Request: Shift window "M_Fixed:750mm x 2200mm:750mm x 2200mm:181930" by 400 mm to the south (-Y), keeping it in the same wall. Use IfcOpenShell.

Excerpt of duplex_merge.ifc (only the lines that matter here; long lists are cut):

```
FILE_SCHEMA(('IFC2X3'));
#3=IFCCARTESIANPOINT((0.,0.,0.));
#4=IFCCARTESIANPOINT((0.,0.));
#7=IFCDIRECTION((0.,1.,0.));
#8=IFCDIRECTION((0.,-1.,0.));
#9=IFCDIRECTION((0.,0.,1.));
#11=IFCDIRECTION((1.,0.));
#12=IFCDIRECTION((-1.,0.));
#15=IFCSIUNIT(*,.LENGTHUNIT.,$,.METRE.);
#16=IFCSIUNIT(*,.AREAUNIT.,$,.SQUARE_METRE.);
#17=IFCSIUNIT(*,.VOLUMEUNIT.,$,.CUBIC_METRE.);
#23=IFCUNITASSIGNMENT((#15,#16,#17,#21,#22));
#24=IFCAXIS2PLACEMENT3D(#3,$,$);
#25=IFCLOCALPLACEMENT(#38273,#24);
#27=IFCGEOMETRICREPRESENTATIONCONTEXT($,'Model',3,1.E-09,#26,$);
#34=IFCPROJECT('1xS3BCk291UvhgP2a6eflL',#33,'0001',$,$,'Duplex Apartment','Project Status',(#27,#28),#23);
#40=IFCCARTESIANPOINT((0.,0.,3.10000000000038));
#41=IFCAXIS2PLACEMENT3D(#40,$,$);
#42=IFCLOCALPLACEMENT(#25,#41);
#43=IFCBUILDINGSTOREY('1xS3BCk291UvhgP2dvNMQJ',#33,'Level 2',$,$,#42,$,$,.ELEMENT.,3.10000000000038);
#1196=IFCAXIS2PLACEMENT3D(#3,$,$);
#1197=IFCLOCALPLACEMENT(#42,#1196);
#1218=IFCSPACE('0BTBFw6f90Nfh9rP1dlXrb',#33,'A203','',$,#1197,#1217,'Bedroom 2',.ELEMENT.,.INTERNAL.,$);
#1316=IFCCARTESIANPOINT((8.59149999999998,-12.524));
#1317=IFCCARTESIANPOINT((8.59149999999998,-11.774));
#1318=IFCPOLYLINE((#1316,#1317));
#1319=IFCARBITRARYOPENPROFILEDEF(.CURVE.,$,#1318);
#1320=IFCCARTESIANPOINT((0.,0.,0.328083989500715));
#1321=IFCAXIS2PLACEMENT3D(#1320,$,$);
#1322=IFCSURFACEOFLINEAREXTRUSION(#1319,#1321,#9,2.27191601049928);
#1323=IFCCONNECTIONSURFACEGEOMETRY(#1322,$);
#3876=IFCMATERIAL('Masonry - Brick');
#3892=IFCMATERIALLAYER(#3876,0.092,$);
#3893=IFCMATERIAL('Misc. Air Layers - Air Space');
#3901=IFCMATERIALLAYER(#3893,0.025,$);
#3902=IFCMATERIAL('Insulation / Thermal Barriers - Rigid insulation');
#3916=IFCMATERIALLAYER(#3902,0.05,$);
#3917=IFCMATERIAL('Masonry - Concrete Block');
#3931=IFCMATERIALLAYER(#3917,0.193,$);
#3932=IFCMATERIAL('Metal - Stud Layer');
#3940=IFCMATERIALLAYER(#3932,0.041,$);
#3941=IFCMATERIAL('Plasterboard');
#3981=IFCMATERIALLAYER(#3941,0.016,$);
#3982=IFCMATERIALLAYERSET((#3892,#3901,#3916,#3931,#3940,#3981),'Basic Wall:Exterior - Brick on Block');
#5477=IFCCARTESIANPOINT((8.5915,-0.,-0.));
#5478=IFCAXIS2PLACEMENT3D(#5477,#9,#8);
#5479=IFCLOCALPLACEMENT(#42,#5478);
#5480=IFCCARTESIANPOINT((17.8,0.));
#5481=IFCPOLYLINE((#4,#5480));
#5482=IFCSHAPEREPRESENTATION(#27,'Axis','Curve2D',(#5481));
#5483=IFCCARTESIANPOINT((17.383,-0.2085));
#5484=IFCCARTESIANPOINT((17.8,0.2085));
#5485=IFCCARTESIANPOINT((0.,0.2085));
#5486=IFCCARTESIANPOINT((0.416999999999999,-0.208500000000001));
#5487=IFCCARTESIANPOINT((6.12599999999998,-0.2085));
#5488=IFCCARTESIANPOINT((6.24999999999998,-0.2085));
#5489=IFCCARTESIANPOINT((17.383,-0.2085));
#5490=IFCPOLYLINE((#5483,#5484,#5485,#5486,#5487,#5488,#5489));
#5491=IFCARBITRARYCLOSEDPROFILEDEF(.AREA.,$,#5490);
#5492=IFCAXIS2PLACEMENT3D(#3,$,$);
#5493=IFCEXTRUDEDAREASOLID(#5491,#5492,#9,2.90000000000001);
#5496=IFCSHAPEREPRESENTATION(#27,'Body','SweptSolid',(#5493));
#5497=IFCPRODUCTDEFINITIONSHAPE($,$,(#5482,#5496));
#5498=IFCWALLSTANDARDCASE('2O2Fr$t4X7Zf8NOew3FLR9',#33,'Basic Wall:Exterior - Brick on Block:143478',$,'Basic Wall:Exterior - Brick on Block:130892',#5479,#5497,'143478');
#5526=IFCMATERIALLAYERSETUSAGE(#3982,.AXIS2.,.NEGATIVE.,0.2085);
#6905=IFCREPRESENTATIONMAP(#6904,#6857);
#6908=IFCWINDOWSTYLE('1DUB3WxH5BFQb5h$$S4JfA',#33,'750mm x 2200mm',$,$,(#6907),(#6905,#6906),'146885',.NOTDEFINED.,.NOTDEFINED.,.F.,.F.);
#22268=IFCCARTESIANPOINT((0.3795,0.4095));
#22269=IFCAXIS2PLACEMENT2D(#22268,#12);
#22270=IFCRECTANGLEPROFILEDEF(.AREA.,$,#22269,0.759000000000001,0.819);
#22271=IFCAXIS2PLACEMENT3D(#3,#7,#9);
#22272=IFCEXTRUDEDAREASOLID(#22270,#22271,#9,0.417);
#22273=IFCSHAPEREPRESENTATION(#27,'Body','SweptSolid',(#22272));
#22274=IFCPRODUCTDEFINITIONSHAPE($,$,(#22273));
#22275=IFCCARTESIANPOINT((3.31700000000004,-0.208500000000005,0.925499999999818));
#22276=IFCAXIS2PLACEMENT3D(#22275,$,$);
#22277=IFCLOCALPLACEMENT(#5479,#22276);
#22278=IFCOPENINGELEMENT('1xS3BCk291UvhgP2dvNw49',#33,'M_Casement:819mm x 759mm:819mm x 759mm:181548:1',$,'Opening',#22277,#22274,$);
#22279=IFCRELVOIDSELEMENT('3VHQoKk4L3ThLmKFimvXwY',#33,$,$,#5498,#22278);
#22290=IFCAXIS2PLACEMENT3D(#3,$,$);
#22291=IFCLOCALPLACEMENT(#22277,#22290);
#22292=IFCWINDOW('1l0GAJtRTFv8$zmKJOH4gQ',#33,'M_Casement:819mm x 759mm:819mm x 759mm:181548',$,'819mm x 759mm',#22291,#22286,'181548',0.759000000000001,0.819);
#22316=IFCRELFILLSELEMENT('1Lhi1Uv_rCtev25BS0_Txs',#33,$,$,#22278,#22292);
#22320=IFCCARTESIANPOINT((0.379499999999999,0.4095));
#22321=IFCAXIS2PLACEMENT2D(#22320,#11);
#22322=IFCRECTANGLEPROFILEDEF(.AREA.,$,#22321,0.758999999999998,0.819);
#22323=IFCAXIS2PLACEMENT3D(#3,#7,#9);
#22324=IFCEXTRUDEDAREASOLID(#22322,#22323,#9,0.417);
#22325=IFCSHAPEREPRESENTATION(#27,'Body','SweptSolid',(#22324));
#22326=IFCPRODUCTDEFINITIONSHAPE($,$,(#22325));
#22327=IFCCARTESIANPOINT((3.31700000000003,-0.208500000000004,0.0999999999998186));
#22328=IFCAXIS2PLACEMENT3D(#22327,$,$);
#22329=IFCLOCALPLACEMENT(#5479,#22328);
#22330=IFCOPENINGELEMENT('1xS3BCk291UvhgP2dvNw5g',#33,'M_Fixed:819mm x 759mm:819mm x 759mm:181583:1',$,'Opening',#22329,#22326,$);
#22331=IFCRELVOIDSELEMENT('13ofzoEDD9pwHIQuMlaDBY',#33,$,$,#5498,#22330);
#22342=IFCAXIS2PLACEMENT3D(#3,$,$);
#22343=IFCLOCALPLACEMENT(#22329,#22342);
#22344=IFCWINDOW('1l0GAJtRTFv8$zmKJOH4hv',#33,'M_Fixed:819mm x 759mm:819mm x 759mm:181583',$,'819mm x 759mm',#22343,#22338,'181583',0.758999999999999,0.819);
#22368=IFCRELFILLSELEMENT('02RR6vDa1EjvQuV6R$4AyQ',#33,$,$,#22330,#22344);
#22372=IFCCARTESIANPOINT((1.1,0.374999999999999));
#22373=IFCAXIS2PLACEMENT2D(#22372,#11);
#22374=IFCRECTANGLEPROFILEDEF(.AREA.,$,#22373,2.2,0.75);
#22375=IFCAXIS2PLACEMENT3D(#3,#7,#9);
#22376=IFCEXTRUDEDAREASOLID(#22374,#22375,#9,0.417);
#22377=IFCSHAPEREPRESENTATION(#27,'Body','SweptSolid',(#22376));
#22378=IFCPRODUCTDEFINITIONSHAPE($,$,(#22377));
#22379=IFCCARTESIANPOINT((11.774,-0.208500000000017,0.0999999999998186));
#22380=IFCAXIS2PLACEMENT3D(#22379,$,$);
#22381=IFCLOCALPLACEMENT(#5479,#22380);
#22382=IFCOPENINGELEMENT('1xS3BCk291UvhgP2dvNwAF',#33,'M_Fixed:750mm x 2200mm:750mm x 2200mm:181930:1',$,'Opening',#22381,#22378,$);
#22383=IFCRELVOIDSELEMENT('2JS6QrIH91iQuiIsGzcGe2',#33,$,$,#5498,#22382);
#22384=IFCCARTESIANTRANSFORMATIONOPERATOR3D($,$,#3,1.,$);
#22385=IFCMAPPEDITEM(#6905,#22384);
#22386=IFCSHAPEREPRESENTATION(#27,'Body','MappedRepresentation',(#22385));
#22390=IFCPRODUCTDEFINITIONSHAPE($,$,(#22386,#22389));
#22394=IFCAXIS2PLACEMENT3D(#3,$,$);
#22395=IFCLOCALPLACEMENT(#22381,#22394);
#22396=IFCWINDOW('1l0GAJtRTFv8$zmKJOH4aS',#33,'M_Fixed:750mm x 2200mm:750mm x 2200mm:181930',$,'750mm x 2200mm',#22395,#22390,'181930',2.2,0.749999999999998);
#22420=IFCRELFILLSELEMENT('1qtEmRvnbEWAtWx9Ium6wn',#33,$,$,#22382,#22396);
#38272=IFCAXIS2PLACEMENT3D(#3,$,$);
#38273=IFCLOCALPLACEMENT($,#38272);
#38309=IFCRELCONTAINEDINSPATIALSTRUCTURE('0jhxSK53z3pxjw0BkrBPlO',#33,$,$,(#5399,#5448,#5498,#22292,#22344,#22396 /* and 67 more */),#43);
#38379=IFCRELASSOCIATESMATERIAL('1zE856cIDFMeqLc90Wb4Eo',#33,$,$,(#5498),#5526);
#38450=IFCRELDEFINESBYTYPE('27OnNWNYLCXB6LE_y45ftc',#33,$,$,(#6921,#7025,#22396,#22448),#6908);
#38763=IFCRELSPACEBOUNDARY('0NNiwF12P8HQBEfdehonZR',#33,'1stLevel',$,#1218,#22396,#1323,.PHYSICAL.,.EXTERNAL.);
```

```python
import numpy as np
import ifcopenshell
import ifcopenshell.api.geometry
import ifcopenshell.util.placement

model = ifcopenshell.open("duplex_merge.ifc")

window = model.by_guid("1l0GAJtRTFv8$zmKJOH4aS")
opening = window.FillsVoids[0].RelatingOpeningElement
wall = opening.VoidsElements[0].RelatingBuildingElement

wall_matrix = ifcopenshell.util.placement.get_local_placement(wall.ObjectPlacement)
shift = wall_matrix[:3, 0] * 0.4
before = ifcopenshell.util.placement.get_local_placement(window.ObjectPlacement)[:3, 3].copy()

# The window is placed relative to its opening, so it follows when the opening moves.
matrix = ifcopenshell.util.placement.get_local_placement(opening.ObjectPlacement)
matrix[:3, 3] += shift
ifcopenshell.api.geometry.edit_object_placement(
    model, product=opening, matrix=matrix, is_si=False, should_transform_children=True
)

# Space boundary surfaces are stored in each space's coordinates; move them too.
for rel in window.ProvidesBoundaries:
    if not rel.ConnectionGeometry:
        continue
    surface = rel.ConnectionGeometry.SurfaceOnRelatingElement
    space_matrix = ifcopenshell.util.placement.get_local_placement(rel.RelatingSpace.ObjectPlacement)
    point = np.array(surface.Position.Location.Coordinates) + space_matrix[:3, :3].T @ shift
    surface.Position = model.createIfcAxis2Placement3D(
        model.createIfcCartesianPoint(point.tolist()), surface.Position.Axis, surface.Position.RefDirection
    )

after = ifcopenshell.util.placement.get_local_placement(window.ObjectPlacement)[:3, 3]
print("window moved by", (after - before).round(3) + 0.0)

model.write("duplex_merge-out.ifc")
```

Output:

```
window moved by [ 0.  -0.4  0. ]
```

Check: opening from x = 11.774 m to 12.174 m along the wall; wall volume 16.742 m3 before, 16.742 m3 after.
